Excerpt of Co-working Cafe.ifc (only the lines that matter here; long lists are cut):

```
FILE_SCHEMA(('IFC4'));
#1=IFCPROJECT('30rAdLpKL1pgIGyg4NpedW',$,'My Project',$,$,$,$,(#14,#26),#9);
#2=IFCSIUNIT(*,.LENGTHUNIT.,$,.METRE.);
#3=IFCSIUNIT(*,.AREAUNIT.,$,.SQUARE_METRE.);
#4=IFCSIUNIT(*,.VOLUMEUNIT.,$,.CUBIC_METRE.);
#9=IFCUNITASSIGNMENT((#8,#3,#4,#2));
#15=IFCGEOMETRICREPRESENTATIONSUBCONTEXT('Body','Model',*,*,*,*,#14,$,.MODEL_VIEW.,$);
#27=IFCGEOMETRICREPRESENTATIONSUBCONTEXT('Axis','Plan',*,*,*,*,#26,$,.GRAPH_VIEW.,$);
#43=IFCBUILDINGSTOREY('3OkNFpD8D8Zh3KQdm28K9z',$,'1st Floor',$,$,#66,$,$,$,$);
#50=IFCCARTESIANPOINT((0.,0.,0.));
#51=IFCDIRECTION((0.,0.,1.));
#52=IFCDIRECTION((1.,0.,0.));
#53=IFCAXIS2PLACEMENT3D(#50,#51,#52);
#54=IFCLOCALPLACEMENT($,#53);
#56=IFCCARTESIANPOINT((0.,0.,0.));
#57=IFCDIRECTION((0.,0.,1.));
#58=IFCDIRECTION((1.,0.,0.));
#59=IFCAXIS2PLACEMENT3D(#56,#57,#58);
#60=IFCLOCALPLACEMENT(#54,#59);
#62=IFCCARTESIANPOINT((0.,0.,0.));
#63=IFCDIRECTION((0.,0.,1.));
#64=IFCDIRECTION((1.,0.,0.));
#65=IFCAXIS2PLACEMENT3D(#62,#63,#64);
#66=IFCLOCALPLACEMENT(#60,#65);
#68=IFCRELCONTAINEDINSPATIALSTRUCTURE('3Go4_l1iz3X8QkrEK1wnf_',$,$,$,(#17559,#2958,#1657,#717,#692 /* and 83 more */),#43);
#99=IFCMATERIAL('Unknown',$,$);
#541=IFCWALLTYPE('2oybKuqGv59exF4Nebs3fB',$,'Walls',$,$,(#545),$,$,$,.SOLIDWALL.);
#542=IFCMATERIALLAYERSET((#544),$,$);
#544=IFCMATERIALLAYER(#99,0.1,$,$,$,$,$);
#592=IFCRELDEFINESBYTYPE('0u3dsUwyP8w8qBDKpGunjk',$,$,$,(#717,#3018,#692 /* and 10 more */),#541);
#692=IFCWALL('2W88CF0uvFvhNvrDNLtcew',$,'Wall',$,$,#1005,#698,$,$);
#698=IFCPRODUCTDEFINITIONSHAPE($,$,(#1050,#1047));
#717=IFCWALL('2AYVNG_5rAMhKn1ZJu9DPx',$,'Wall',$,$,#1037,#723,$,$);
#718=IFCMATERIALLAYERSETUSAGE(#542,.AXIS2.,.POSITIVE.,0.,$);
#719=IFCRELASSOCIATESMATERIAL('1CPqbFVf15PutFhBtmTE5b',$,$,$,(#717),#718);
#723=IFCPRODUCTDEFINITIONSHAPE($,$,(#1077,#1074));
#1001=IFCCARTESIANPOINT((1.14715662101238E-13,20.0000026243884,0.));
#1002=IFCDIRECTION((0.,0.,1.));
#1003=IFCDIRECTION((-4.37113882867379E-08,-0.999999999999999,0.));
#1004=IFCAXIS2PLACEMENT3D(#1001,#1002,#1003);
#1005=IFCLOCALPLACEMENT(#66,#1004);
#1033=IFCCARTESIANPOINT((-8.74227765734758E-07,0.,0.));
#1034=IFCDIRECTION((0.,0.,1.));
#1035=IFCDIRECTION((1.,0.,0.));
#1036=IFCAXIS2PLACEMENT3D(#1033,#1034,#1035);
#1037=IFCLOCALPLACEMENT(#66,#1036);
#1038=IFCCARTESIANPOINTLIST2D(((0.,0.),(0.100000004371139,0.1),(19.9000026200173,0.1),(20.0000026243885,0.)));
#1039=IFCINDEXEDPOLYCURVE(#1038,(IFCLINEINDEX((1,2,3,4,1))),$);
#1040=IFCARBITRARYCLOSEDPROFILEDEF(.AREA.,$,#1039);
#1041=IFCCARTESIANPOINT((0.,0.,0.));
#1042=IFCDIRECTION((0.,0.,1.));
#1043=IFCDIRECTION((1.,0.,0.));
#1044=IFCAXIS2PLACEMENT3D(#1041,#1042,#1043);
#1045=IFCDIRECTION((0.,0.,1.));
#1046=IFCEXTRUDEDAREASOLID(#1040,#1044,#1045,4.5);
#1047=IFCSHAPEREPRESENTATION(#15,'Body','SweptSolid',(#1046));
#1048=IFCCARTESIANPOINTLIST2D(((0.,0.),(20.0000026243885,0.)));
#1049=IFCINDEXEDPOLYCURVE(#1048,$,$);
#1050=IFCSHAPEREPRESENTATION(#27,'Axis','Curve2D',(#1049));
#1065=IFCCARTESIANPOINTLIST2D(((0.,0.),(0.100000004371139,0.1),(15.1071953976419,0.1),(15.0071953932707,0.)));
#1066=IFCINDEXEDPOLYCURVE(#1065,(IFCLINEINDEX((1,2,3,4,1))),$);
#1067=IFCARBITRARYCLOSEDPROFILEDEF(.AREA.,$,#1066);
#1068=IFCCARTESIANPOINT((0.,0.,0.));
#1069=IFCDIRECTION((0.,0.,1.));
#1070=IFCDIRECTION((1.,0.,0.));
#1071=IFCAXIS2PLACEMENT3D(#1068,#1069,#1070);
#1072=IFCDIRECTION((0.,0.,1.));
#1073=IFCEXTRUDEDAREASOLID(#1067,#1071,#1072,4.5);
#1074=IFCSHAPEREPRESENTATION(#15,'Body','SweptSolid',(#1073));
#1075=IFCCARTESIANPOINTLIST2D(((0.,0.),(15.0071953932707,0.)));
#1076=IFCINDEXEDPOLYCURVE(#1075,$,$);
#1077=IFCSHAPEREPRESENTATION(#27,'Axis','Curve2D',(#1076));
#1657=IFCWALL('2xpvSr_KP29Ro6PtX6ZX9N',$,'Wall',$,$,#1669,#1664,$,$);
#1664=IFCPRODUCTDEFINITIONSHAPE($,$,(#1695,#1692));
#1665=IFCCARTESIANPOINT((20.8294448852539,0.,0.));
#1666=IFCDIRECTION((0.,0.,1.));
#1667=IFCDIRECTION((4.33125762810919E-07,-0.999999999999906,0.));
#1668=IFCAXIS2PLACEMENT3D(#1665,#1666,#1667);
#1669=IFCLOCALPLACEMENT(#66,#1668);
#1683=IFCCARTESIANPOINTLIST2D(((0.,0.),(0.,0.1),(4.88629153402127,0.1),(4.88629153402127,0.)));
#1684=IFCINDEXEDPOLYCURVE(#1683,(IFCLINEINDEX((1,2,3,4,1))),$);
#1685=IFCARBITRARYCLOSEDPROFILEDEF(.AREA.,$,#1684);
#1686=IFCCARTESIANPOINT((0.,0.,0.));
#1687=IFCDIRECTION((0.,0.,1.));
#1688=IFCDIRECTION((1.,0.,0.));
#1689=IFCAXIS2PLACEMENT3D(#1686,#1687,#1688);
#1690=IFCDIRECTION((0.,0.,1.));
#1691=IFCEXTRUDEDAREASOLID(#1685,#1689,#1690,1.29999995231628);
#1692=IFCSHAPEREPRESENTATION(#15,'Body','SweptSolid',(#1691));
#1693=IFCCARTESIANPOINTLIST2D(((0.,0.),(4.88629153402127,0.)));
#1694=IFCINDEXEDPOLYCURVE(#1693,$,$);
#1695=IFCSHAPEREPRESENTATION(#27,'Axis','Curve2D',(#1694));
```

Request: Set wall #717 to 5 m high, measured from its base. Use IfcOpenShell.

```python
import ifcopenshell
import ifcopenshell.geom
import ifcopenshell.util.representation
import ifcopenshell.util.shape
import ifcopenshell.util.unit

model = ifcopenshell.open("Co-working Cafe.ifc")
unit_scale = ifcopenshell.util.unit.calculate_unit_scale(model)
settings = ifcopenshell.geom.settings()


def volume(element):
    """Net volume in cubic metres, openings subtracted."""
    shape = ifcopenshell.geom.create_shape(settings, element)
    return ifcopenshell.util.shape.get_volume(shape.geometry)


wall = model.by_guid("2AYVNG_5rAMhKn1ZJu9DPx")
before = volume(wall)

body = ifcopenshell.util.representation.get_representation(wall, "Model", "Body")
solid = body.Items[0]
old_height = solid.Depth
solid.Depth = 5 / unit_scale
after = volume(wall)

print(f"height {old_height:g} -> {solid.Depth:g}, volume {before:.3f} -> {after:.3f} m3")

model.write("Co-working Cafe_edited.ifc")
```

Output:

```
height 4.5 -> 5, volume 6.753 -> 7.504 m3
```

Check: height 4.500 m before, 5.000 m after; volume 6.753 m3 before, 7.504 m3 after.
